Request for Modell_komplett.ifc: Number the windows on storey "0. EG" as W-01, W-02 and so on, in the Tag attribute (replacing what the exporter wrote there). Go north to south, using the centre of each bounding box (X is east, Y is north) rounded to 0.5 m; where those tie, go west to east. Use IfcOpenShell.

First a look at what the model holds.

```python
import ifcopenshell
import ifcopenshell.util.element
import ifcopenshell.util.placement

model = ifcopenshell.open("Modell_komplett.ifc")
print(model.schema)
storey = next(s for s in model.by_type("IfcBuildingStorey") if s.Name == "0. EG")
windows = [e for e in ifcopenshell.util.element.get_decomposition(storey) if e.is_a("IfcWindow")]
for e in sorted(windows, key=lambda e: e.id()):
    origin = ifcopenshell.util.placement.get_local_placement(e.ObjectPlacement)[:3, 3]
    print(e.id(), e.Tag, e.Name, origin.round(2) + 0.0, sep=" | ")
```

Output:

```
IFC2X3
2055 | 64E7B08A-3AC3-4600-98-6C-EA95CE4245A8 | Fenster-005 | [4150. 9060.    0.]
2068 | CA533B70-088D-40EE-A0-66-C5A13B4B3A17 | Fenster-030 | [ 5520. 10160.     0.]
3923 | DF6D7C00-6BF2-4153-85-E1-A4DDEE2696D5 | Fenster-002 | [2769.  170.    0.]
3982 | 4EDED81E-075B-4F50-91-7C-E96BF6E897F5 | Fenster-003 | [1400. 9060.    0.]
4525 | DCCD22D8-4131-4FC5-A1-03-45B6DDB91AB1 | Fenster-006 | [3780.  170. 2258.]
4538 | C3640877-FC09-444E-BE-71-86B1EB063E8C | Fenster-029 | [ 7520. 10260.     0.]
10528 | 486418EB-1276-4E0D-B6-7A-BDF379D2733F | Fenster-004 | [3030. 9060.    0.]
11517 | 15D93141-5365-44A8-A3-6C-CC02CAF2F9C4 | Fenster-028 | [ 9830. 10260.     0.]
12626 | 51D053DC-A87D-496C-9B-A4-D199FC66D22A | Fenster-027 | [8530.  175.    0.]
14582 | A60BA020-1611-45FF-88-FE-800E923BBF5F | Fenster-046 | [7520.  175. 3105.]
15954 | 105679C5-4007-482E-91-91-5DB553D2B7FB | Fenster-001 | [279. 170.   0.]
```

```python
import ifcopenshell
import ifcopenshell.geom
import ifcopenshell.util.element
import ifcopenshell.util.shape

model = ifcopenshell.open("Modell_komplett.ifc")
settings = ifcopenshell.geom.settings()
settings.set("use-world-coords", True)


def centre(element):
    shape = ifcopenshell.geom.create_shape(settings, element)
    return ifcopenshell.util.shape.get_bbox_centroid(shape.geometry)


storey = next(s for s in model.by_type("IfcBuildingStorey") if s.Name == "0. EG")
windows = [e for e in ifcopenshell.util.element.get_decomposition(storey) if e.is_a("IfcWindow")]

# Insertion points can sit at a corner or the storey origin, so sort by the geometry (in metres).
centres = {e: centre(e) for e in windows}
windows.sort(key=lambda e: (-round(centres[e][1] / 0.5), centres[e][0]))

for i, e in enumerate(windows, start=1):
    number = f"W-{i:02d}"
    e.Tag = number
    print(e.id(), number)

model.write("Modell_komplett_rev.ifc")
```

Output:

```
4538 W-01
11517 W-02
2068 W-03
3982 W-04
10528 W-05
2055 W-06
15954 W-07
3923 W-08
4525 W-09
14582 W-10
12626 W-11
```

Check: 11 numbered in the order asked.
